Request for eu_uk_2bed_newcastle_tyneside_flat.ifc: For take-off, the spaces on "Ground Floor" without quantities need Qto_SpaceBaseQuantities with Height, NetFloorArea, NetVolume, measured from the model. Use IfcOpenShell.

First a look at what the model holds.

```python
import ifcopenshell
import ifcopenshell.util.element
import ifcopenshell.util.unit

model = ifcopenshell.open("eu_uk_2bed_newcastle_tyneside_flat.ifc")
print(model.schema)
for unit_type in ("LENGTHUNIT", "AREAUNIT", "VOLUMEUNIT"):
    print(unit_type, ifcopenshell.util.unit.calculate_unit_scale(model, unit_type))
storey = next(s for s in model.by_type("IfcBuildingStorey") if s.Name == "Ground Floor")
spaces = [e for e in ifcopenshell.util.element.get_decomposition(storey) if e.is_a("IfcSpace")]
for e in sorted(spaces, key=lambda e: e.id()):
    print(e.id(), e.is_a(), e.Name, list(ifcopenshell.util.element.get_psets(e, qtos_only=True)), sep=" | ")
```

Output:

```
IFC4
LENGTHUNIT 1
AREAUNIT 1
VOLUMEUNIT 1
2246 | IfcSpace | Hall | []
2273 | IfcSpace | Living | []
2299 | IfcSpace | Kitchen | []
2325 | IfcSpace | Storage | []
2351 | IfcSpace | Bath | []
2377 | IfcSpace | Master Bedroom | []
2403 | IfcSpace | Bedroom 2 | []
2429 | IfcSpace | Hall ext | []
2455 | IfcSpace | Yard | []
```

```python
import ifcopenshell
import ifcopenshell.api.pset
import ifcopenshell.geom
import ifcopenshell.util.element
import ifcopenshell.util.shape
import ifcopenshell.util.unit

model = ifcopenshell.open("eu_uk_2bed_newcastle_tyneside_flat.ifc")
unit_scale = ifcopenshell.util.unit.calculate_unit_scale(model)
area_scale = ifcopenshell.util.unit.calculate_unit_scale(model, "AREAUNIT")
volume_scale = ifcopenshell.util.unit.calculate_unit_scale(model, "VOLUMEUNIT")
settings = ifcopenshell.geom.settings()

storey = next(s for s in model.by_type("IfcBuildingStorey") if s.Name == "Ground Floor")
spaces = [e for e in ifcopenshell.util.element.get_decomposition(storey) if e.is_a("IfcSpace")]

for e in sorted(spaces, key=lambda e: e.id()):
    if ifcopenshell.util.element.get_psets(e, qtos_only=True, should_inherit=False):
        continue
    # Geometry comes back in metres, in the element's own axes.
    shape = ifcopenshell.geom.create_shape(settings, e)
    values = {
        "Height": ifcopenshell.util.shape.get_z(shape.geometry) / unit_scale,
        "NetFloorArea": ifcopenshell.util.shape.get_footprint_area(shape.geometry) / area_scale,
        "NetVolume": ifcopenshell.util.shape.get_volume(shape.geometry) / volume_scale,
    }
    qto = ifcopenshell.api.pset.add_qto(model, product=e, name="Qto_SpaceBaseQuantities")
    ifcopenshell.api.pset.edit_qto(model, qto=qto, properties=values)
    print(e.id(), {k: round(v, 3) for k, v in values.items()})

model.write("eu_uk_2bed_newcastle_tyneside_flat_updated.ifc")
```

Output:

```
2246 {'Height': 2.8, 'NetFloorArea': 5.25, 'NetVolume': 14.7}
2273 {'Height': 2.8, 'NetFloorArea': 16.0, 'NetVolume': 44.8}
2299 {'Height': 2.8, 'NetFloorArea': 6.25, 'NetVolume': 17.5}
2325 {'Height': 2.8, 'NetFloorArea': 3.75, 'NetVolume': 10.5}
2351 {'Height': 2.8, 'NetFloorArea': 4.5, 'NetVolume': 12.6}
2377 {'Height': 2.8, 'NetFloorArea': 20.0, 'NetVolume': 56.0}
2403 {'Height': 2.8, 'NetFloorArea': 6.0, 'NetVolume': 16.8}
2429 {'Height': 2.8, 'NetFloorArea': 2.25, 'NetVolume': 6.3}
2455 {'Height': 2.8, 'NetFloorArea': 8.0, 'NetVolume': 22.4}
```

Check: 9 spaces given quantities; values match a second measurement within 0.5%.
